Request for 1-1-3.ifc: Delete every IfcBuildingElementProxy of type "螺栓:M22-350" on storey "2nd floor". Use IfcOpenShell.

First a look at what the model holds.

```python
import ifcopenshell
import ifcopenshell.util.element

model = ifcopenshell.open("1-1-3.ifc")
print(model.schema)
storey = next(s for s in model.by_type("IfcBuildingStorey") if s.Name == "2nd floor")
proxies = [e for e in ifcopenshell.util.element.get_decomposition(storey) if e.is_a("IfcBuildingElementProxy")]
seen = {}
for e in proxies:
    element_type = ifcopenshell.util.element.get_type(e)
    name = element_type.Name if element_type not in (None, e) else None
    seen[name] = seen.get(name, 0) + 1
for name, count in sorted(seen.items(), key=str):
    print(count, "x", name)
```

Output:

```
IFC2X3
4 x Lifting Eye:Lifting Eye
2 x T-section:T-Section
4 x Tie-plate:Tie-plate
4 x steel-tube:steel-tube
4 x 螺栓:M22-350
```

```python
import ifcopenshell
import ifcopenshell.api.root
import ifcopenshell.util.element

model = ifcopenshell.open("1-1-3.ifc")

storey = next(s for s in model.by_type("IfcBuildingStorey") if s.Name == "2nd floor")
proxies = [e for e in ifcopenshell.util.element.get_decomposition(storey) if e.is_a("IfcBuildingElementProxy")]
targets = [e for e in proxies if (t := ifcopenshell.util.element.get_type(e)) not in (None, e) and t.Name == "螺栓:M22-350"]

for e in targets:
    ifcopenshell.api.root.remove_product(model, product=e)
print(len(targets), "removed")

model.write("1-1-3_edited.ifc")
```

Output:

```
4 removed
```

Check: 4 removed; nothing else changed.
